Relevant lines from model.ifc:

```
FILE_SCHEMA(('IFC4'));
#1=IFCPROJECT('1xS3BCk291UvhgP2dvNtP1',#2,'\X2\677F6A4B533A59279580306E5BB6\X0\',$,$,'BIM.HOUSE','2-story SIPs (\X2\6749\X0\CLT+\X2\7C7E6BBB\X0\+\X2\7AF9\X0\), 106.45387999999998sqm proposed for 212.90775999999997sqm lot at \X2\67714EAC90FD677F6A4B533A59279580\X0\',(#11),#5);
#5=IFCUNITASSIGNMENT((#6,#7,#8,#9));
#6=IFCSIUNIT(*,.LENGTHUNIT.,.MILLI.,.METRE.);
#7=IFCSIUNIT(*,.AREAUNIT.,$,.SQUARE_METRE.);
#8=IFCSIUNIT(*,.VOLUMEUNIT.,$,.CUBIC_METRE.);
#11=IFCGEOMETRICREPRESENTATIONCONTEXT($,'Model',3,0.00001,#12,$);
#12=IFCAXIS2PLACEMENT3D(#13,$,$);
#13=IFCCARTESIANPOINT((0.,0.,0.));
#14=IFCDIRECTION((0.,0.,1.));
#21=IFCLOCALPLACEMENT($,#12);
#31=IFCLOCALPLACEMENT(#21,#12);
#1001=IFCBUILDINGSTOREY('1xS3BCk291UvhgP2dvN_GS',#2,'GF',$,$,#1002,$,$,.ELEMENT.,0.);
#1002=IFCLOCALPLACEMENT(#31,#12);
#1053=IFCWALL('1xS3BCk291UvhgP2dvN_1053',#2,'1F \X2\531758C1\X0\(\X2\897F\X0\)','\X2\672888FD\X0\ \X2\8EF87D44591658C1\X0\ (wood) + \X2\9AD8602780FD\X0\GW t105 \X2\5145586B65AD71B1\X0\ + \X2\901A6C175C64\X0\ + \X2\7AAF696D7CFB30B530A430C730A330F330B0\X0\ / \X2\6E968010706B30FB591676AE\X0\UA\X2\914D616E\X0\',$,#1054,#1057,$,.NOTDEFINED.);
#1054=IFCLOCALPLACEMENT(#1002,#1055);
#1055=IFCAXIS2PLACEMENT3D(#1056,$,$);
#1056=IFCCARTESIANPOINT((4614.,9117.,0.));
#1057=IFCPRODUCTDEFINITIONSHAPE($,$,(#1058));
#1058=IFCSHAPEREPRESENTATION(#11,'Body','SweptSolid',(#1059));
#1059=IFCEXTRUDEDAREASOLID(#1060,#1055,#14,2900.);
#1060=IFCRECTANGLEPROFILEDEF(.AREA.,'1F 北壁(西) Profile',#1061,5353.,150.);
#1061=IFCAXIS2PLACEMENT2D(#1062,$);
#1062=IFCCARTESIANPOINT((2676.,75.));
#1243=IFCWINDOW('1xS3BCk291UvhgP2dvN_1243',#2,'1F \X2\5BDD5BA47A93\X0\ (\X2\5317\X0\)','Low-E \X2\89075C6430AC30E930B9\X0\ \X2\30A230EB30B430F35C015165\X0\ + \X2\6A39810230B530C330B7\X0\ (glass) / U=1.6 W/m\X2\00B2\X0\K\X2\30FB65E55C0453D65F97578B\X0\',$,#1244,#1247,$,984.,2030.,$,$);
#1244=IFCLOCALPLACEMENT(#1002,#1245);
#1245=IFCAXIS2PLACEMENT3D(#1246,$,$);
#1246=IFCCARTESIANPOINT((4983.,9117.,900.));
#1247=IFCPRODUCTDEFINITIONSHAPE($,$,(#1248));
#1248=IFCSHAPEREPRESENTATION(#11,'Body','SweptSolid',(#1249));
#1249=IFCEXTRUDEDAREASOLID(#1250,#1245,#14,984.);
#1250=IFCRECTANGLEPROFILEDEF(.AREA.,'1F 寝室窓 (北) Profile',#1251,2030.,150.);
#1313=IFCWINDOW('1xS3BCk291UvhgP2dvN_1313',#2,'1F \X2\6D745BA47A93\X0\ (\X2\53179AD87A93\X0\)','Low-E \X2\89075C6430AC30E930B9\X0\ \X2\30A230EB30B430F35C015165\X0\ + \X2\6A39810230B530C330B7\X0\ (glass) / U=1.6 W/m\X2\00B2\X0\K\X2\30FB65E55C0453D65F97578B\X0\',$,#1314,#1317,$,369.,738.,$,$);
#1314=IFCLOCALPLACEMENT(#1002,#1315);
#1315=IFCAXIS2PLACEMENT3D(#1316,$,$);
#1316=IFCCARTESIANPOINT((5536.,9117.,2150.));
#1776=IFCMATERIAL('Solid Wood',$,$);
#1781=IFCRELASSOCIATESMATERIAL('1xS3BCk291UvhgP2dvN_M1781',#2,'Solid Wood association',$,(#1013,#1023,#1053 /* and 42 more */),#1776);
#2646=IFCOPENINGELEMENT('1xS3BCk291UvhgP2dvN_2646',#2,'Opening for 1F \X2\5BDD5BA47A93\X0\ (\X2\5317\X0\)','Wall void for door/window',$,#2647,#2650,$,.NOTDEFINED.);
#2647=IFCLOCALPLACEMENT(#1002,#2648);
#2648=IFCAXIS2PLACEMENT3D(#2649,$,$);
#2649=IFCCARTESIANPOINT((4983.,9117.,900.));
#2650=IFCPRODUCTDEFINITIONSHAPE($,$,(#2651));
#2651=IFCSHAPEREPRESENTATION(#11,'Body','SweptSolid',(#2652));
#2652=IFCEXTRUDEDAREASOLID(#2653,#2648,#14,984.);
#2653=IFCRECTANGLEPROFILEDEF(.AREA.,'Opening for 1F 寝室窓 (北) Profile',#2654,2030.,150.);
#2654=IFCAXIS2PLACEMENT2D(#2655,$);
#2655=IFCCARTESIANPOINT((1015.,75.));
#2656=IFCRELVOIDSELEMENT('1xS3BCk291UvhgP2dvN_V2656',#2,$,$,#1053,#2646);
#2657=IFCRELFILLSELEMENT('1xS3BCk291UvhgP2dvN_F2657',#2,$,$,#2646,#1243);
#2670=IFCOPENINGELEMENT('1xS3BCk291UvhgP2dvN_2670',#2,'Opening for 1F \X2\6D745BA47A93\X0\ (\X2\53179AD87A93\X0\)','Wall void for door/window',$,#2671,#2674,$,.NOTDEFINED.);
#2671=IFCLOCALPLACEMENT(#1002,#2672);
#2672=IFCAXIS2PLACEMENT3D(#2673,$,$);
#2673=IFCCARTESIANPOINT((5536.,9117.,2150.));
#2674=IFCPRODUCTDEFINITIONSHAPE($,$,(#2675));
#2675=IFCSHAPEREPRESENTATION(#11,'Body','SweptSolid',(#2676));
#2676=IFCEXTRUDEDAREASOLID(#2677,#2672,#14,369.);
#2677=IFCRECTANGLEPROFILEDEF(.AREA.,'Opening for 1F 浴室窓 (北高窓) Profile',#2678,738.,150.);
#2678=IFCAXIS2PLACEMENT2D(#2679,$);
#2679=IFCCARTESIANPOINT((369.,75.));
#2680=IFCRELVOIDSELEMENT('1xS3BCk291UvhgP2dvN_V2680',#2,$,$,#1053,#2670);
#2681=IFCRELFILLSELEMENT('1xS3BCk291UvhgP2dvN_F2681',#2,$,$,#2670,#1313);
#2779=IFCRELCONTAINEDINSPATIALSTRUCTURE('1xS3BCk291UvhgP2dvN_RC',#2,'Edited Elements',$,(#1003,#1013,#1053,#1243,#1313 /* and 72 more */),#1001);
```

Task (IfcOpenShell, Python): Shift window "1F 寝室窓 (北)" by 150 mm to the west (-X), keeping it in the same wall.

```python
import ifcopenshell
import ifcopenshell.api.geometry
import ifcopenshell.util.placement
import ifcopenshell.util.unit

model = ifcopenshell.open("model.ifc")
unit_scale = ifcopenshell.util.unit.calculate_unit_scale(model)

window = model.by_id(1243)
opening = window.FillsVoids[0].RelatingOpeningElement
wall = opening.VoidsElements[0].RelatingBuildingElement

wall_matrix = ifcopenshell.util.placement.get_local_placement(wall.ObjectPlacement)
shift = wall_matrix[:3, 0] * -0.15 / unit_scale
before = ifcopenshell.util.placement.get_local_placement(window.ObjectPlacement)[:3, 3].copy()

# The window is not placed relative to its opening, so move both.
for product in (opening, window):
    matrix = ifcopenshell.util.placement.get_local_placement(product.ObjectPlacement)
    matrix[:3, 3] += shift
    ifcopenshell.api.geometry.edit_object_placement(model, product=product, matrix=matrix, is_si=False)

after = ifcopenshell.util.placement.get_local_placement(window.ObjectPlacement)[:3, 3]
print("window moved by", (after - before).round(3) + 0.0)

model.write("model-out.ifc")
```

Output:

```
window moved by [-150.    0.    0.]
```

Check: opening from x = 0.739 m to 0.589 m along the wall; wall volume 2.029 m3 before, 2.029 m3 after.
